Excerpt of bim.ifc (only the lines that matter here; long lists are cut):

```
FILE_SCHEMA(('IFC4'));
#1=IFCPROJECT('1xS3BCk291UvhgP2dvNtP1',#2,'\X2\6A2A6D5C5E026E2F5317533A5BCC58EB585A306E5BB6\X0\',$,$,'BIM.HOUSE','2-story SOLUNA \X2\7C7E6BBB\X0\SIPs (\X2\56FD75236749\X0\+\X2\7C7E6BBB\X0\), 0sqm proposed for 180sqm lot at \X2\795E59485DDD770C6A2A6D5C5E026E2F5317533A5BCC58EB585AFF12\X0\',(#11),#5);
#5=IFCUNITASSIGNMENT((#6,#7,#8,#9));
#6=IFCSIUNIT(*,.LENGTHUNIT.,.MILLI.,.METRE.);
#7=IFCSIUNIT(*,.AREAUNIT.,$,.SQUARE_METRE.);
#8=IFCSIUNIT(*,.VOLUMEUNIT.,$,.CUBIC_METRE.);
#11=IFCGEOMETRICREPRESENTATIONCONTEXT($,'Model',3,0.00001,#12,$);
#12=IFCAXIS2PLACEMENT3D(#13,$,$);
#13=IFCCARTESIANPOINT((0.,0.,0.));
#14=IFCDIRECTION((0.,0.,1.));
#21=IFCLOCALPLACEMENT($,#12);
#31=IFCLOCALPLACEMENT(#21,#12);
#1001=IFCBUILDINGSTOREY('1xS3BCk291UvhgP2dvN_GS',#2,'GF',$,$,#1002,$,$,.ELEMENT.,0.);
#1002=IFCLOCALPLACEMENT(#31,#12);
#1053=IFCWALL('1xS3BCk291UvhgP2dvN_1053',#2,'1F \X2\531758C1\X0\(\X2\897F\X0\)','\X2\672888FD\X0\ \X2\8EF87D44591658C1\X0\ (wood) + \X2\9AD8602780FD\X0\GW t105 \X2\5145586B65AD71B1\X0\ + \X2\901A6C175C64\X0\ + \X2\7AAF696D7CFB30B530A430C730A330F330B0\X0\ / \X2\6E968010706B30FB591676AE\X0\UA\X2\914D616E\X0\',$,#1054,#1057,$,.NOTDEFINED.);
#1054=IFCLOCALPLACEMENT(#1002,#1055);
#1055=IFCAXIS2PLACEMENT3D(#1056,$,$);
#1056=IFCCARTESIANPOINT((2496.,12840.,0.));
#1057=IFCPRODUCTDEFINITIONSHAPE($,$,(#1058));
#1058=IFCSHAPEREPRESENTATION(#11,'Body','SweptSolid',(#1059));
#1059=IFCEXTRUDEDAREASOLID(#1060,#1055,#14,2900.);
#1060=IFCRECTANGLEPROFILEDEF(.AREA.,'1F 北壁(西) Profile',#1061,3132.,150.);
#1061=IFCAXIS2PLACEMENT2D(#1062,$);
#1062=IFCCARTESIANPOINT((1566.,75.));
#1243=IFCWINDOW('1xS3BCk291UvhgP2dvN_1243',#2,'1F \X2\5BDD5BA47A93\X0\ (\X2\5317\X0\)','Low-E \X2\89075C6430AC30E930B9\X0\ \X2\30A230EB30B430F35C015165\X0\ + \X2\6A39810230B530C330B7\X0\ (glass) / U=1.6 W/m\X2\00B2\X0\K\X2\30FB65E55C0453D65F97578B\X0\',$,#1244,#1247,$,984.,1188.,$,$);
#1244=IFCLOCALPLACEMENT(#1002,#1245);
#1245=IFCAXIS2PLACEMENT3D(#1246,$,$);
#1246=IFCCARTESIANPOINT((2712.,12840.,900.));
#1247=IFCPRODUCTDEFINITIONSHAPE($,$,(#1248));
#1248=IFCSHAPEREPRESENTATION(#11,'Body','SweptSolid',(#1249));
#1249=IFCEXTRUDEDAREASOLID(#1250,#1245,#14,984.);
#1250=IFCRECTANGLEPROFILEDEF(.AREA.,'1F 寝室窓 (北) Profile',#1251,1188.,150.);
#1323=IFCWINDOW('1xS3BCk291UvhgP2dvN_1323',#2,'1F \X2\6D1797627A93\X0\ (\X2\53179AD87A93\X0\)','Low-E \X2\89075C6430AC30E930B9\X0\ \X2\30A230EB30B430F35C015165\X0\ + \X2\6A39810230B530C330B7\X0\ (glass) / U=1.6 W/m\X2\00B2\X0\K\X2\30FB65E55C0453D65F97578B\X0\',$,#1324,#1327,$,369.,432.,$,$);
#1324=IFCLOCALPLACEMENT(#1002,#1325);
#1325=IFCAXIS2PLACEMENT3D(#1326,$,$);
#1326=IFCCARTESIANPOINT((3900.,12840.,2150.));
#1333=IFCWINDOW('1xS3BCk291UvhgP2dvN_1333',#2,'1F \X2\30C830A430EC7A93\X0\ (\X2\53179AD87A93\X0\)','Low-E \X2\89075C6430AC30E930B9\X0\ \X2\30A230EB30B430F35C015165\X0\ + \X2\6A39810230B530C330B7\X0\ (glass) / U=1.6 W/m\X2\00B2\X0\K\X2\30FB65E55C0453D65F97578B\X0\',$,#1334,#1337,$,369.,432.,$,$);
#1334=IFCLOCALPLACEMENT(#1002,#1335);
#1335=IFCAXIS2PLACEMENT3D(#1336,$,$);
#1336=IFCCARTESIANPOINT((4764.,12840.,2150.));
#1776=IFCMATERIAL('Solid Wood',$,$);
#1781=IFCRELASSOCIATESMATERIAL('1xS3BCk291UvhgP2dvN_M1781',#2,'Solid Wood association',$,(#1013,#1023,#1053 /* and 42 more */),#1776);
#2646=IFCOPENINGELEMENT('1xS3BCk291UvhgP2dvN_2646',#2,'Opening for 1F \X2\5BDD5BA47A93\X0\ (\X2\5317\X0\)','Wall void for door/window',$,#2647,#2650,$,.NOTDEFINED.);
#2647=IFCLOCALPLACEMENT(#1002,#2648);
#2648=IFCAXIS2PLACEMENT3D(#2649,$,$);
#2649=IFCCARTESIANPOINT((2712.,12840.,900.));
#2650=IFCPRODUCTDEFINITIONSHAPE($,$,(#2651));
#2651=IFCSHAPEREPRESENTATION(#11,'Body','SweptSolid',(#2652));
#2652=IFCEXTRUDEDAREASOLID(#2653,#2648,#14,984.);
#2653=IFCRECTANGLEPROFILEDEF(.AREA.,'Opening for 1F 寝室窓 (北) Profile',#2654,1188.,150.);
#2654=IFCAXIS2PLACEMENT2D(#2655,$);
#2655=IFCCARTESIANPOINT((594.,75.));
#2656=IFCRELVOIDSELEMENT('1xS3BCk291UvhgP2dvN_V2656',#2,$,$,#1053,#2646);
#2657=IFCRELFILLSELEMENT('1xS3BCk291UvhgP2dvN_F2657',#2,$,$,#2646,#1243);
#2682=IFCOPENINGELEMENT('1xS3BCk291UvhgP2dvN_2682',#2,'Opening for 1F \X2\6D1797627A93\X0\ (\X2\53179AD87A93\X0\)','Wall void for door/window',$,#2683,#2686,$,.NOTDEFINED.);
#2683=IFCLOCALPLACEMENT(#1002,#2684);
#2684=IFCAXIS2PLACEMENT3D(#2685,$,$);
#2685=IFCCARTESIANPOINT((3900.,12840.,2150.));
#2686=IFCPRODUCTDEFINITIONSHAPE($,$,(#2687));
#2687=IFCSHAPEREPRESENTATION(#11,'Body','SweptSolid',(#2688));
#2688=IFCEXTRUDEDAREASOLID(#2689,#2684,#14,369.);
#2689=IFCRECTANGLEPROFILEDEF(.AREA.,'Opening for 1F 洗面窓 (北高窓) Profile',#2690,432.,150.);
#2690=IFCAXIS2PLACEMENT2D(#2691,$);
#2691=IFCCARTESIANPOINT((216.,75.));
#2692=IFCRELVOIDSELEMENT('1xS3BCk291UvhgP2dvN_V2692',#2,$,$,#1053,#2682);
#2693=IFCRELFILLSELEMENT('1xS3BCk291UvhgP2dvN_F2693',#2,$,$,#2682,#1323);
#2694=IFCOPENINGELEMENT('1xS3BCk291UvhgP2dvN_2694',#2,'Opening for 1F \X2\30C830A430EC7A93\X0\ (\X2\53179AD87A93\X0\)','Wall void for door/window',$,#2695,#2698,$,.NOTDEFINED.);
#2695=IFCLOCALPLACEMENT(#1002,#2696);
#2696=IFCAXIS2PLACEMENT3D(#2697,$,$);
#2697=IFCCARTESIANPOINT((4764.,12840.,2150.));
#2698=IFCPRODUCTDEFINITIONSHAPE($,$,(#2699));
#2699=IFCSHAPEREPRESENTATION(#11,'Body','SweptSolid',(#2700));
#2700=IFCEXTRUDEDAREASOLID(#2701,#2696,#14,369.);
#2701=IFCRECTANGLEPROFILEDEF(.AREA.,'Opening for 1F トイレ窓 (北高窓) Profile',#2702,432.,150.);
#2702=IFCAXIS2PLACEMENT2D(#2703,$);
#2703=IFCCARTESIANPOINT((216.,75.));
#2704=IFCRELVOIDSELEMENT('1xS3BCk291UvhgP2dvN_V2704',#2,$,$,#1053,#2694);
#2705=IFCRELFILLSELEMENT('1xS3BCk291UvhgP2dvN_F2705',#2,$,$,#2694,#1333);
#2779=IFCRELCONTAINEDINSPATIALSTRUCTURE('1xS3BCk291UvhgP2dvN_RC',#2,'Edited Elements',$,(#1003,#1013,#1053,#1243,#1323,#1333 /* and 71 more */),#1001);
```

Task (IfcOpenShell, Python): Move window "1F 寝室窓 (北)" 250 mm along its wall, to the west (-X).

```python
import ifcopenshell
import ifcopenshell.api.geometry
import ifcopenshell.util.placement
import ifcopenshell.util.unit

model = ifcopenshell.open("bim.ifc")
unit_scale = ifcopenshell.util.unit.calculate_unit_scale(model)

window = model.by_guid("1xS3BCk291UvhgP2dvN_1243")
opening = window.FillsVoids[0].RelatingOpeningElement
wall = opening.VoidsElements[0].RelatingBuildingElement

wall_matrix = ifcopenshell.util.placement.get_local_placement(wall.ObjectPlacement)
shift = wall_matrix[:3, 0] * -0.25 / unit_scale
before = ifcopenshell.util.placement.get_local_placement(window.ObjectPlacement)[:3, 3].copy()

# The window is not placed relative to its opening, so move both.
for product in (opening, window):
    matrix = ifcopenshell.util.placement.get_local_placement(product.ObjectPlacement)
    matrix[:3, 3] += shift
    ifcopenshell.api.geometry.edit_object_placement(model, product=product, matrix=matrix, is_si=False)

after = ifcopenshell.util.placement.get_local_placement(window.ObjectPlacement)[:3, 3]
print("window moved by", (after - before).round(3) + 0.0)

model.write("bim_edited.ifc")
```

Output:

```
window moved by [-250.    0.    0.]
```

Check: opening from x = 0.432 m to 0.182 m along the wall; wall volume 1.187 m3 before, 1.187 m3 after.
